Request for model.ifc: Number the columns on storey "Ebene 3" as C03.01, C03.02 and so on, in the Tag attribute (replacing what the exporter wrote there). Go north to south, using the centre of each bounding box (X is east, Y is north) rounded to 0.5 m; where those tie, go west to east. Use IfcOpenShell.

First a look at what the model holds.

```python
import ifcopenshell
import ifcopenshell.util.element
import ifcopenshell.util.placement

model = ifcopenshell.open("model.ifc")
print(model.schema)
storey = next(s for s in model.by_type("IfcBuildingStorey") if s.Name == "Ebene 3")
columns = [e for e in ifcopenshell.util.element.get_decomposition(storey) if e.is_a("IfcColumn")]
for e in sorted(columns, key=lambda e: e.id()):
    origin = ifcopenshell.util.placement.get_local_placement(e.ObjectPlacement)[:3, 3]
    print(e.id(), e.Tag, e.Name, origin.round(2) + 0.0, sep=" | ")
```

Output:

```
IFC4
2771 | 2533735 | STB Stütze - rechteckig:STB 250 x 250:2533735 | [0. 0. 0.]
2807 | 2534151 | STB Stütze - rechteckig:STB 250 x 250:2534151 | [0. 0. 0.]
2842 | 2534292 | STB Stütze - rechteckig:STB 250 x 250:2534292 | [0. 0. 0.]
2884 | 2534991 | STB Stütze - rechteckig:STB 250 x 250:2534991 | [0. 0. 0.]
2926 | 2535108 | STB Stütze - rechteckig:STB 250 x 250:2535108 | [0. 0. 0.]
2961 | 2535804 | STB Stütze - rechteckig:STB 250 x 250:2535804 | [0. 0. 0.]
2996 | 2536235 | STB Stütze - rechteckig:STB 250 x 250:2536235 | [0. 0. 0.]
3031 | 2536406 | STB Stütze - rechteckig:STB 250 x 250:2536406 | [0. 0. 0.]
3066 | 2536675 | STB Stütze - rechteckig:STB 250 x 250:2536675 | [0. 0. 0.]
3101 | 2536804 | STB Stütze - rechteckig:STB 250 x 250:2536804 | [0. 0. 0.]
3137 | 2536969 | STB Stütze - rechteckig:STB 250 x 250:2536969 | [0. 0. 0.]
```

```python
import ifcopenshell
import ifcopenshell.geom
import ifcopenshell.util.element
import ifcopenshell.util.shape

model = ifcopenshell.open("model.ifc")
settings = ifcopenshell.geom.settings()
settings.set("use-world-coords", True)


def centre(element):
    shape = ifcopenshell.geom.create_shape(settings, element)
    return ifcopenshell.util.shape.get_bbox_centroid(shape.geometry)


storey = next(s for s in model.by_type("IfcBuildingStorey") if s.Name == "Ebene 3")
columns = [e for e in ifcopenshell.util.element.get_decomposition(storey) if e.is_a("IfcColumn")]

# Insertion points can sit at a corner or the storey origin, so sort by the geometry (in metres).
centres = {e: centre(e) for e in columns}
columns.sort(key=lambda e: (-round(centres[e][1] / 0.5), centres[e][0]))

for i, e in enumerate(columns, start=1):
    number = f"C03.{i:02d}"
    e.Tag = number
    print(e.id(), number)

model.write("model_updated.ifc")
```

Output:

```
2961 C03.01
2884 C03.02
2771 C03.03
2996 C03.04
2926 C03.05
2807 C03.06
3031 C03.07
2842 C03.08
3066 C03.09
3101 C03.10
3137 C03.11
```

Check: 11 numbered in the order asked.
